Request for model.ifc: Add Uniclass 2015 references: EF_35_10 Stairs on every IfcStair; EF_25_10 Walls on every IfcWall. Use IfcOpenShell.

First a look at what the model holds.

```python
import ifcopenshell

model = ifcopenshell.open("model.ifc")
print(model.schema)
print("classifications:", [c.Name for c in model.by_type("IfcClassification")])
for ifc_class in ("IfcDoor", "IfcRoof", "IfcStair", "IfcWall", "IfcWindow"):
    print(ifc_class, len(model.by_type(ifc_class)))
```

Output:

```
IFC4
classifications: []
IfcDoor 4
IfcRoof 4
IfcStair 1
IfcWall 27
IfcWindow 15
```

```python
import ifcopenshell
import ifcopenshell.api.classification

model = ifcopenshell.open("model.ifc")

system = ifcopenshell.api.classification.add_classification(model, classification="Uniclass 2015")

codes = {
    "IfcStair": ("EF_35_10", "Stairs"),
    "IfcWall": ("EF_25_10", "Walls"),
}
for ifc_class, (code, name) in codes.items():
    products = model.by_type(ifc_class)
    ifcopenshell.api.classification.add_reference(
        model, products=products, classification=system, identification=code, name=name
    )
    print(code, len(products))

model.write("model_v2.ifc")
```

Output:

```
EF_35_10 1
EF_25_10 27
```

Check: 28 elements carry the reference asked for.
